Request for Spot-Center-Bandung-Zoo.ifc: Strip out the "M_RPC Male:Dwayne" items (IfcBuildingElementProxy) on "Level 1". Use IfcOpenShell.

First a look at what the model holds.

```python
import ifcopenshell
import ifcopenshell.util.element

model = ifcopenshell.open("Spot-Center-Bandung-Zoo.ifc")
print(model.schema)
storey = next(s for s in model.by_type("IfcBuildingStorey") if s.Name == "Level 1")
proxies = [e for e in ifcopenshell.util.element.get_decomposition(storey) if e.is_a("IfcBuildingElementProxy")]
seen = {}
for e in proxies:
    element_type = ifcopenshell.util.element.get_type(e)
    name = element_type.Name if element_type not in (None, e) else None
    seen[name] = seen.get(name, 0) + 1
for name, count in sorted(seen.items(), key=str):
    print(count, "x", name)
```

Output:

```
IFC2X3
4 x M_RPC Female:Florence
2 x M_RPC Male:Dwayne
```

```python
import ifcopenshell
import ifcopenshell.api.root
import ifcopenshell.util.element

model = ifcopenshell.open("Spot-Center-Bandung-Zoo.ifc")

storey = next(s for s in model.by_type("IfcBuildingStorey") if s.Name == "Level 1")
proxies = [e for e in ifcopenshell.util.element.get_decomposition(storey) if e.is_a("IfcBuildingElementProxy")]
targets = [e for e in proxies if (t := ifcopenshell.util.element.get_type(e)) not in (None, e) and t.Name == "M_RPC Male:Dwayne"]

for e in targets:
    ifcopenshell.api.root.remove_product(model, product=e)
print(len(targets), "removed")

model.write("Spot-Center-Bandung-Zoo_edited.ifc")
```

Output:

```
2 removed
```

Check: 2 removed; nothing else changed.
